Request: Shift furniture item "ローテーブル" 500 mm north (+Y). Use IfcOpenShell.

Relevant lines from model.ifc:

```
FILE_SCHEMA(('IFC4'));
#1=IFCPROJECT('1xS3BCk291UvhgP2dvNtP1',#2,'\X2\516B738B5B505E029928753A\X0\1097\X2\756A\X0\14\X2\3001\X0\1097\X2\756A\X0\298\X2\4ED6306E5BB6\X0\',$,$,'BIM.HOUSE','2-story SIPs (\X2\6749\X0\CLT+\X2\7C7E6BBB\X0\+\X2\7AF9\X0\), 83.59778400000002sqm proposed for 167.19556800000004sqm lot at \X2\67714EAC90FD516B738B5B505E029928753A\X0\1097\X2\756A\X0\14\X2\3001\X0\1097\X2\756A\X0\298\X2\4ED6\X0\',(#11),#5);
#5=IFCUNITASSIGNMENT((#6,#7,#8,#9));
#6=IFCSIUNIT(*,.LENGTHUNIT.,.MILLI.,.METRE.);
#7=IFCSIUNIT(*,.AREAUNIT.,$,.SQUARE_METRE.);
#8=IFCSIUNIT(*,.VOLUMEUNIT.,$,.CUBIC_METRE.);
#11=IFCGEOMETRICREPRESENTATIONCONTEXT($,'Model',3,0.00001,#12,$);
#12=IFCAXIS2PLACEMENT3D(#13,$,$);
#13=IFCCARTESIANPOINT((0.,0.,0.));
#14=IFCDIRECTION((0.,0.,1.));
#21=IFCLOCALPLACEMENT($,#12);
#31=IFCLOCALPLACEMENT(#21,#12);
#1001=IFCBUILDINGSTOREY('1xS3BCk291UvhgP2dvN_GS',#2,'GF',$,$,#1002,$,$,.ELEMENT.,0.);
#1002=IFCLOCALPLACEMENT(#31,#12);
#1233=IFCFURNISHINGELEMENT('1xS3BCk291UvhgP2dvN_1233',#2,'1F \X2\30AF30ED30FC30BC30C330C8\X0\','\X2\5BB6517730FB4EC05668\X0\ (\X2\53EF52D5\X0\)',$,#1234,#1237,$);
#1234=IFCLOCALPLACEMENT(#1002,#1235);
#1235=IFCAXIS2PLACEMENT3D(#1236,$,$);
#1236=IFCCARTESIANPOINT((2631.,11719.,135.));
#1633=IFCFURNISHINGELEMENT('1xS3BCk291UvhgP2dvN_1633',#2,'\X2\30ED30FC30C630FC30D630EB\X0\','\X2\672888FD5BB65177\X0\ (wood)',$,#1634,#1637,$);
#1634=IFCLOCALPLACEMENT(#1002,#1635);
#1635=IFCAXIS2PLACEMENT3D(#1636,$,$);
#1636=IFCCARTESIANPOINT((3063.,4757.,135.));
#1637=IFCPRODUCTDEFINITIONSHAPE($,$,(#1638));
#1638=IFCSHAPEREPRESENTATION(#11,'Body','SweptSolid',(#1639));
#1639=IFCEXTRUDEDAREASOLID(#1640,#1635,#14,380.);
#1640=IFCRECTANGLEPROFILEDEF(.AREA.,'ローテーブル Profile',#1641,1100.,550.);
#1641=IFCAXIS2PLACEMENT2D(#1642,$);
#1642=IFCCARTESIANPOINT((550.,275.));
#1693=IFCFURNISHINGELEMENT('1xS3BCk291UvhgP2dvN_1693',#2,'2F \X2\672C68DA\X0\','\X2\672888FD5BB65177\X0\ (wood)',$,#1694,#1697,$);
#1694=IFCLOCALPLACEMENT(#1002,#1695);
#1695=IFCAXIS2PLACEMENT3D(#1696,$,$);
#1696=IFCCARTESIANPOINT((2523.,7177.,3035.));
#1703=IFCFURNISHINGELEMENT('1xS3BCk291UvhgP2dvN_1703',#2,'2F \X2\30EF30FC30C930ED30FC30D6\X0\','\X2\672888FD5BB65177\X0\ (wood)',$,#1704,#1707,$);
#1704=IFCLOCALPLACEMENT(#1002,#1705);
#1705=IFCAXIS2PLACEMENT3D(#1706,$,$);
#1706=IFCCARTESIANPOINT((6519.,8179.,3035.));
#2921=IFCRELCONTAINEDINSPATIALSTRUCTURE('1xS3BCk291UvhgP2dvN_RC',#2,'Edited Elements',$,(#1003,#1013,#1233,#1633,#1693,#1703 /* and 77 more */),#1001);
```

```python
import ifcopenshell
import ifcopenshell.api.geometry
import ifcopenshell.util.placement
import ifcopenshell.util.unit

model = ifcopenshell.open("model.ifc")
unit_scale = ifcopenshell.util.unit.calculate_unit_scale(model)

item = model.by_guid("1xS3BCk291UvhgP2dvN_1633")
matrix = ifcopenshell.util.placement.get_local_placement(item.ObjectPlacement)
matrix[1, 3] += 0.5 / unit_scale
ifcopenshell.api.geometry.edit_object_placement(model, product=item, matrix=matrix, is_si=False)

print(ifcopenshell.util.placement.get_local_placement(item.ObjectPlacement).round(3) + 0.0)

model.write("model_v2.ifc")
```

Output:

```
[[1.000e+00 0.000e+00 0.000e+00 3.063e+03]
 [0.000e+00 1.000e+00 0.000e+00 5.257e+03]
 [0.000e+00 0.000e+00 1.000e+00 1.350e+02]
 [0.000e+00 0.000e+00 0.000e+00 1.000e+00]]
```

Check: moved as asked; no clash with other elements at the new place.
